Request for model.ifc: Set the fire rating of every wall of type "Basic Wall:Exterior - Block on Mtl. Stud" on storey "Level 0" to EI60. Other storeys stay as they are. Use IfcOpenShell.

First a look at what the model holds.

```python
import ifcopenshell
import ifcopenshell.util.element

model = ifcopenshell.open("model.ifc")
print(model.schema)
storey = next(s for s in model.by_type("IfcBuildingStorey") if s.Name == "Level 0")
walls = [e for e in ifcopenshell.util.element.get_decomposition(storey) if e.is_a("IfcWall")]
seen = {}
for e in walls:
    element_type = ifcopenshell.util.element.get_type(e)
    key = (element_type.Name if element_type != e and element_type else None, ifcopenshell.util.element.get_pset(e, "Pset_WallCommon", "FireRating"))
    seen[key] = seen.get(key, 0) + 1
for (name, value), count in sorted(seen.items(), key=str):
    print(count, "x", name, "|", value)
```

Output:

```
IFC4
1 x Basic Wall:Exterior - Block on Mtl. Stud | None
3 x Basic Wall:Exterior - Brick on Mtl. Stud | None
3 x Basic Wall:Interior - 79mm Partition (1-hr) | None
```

```python
import ifcopenshell
import ifcopenshell.api.pset
import ifcopenshell.util.element

model = ifcopenshell.open("model.ifc")

storey = next(s for s in model.by_type("IfcBuildingStorey") if s.Name == "Level 0")
walls = [e for e in ifcopenshell.util.element.get_decomposition(storey) if e.is_a("IfcWall")]

count = 0
for e in walls:
    element_type = ifcopenshell.util.element.get_type(e)
    if element_type in (None, e) or element_type.Name != "Basic Wall:Exterior - Block on Mtl. Stud":
        continue
    # add_pset returns the element's existing set when there is one.
    pset = ifcopenshell.api.pset.add_pset(model, product=e, name="Pset_WallCommon")
    ifcopenshell.api.pset.edit_pset(model, pset=pset, properties={"FireRating": "EI60"})
    count += 1

print(count, "walls updated")

model.write("model-out.ifc")
```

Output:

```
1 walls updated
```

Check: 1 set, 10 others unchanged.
